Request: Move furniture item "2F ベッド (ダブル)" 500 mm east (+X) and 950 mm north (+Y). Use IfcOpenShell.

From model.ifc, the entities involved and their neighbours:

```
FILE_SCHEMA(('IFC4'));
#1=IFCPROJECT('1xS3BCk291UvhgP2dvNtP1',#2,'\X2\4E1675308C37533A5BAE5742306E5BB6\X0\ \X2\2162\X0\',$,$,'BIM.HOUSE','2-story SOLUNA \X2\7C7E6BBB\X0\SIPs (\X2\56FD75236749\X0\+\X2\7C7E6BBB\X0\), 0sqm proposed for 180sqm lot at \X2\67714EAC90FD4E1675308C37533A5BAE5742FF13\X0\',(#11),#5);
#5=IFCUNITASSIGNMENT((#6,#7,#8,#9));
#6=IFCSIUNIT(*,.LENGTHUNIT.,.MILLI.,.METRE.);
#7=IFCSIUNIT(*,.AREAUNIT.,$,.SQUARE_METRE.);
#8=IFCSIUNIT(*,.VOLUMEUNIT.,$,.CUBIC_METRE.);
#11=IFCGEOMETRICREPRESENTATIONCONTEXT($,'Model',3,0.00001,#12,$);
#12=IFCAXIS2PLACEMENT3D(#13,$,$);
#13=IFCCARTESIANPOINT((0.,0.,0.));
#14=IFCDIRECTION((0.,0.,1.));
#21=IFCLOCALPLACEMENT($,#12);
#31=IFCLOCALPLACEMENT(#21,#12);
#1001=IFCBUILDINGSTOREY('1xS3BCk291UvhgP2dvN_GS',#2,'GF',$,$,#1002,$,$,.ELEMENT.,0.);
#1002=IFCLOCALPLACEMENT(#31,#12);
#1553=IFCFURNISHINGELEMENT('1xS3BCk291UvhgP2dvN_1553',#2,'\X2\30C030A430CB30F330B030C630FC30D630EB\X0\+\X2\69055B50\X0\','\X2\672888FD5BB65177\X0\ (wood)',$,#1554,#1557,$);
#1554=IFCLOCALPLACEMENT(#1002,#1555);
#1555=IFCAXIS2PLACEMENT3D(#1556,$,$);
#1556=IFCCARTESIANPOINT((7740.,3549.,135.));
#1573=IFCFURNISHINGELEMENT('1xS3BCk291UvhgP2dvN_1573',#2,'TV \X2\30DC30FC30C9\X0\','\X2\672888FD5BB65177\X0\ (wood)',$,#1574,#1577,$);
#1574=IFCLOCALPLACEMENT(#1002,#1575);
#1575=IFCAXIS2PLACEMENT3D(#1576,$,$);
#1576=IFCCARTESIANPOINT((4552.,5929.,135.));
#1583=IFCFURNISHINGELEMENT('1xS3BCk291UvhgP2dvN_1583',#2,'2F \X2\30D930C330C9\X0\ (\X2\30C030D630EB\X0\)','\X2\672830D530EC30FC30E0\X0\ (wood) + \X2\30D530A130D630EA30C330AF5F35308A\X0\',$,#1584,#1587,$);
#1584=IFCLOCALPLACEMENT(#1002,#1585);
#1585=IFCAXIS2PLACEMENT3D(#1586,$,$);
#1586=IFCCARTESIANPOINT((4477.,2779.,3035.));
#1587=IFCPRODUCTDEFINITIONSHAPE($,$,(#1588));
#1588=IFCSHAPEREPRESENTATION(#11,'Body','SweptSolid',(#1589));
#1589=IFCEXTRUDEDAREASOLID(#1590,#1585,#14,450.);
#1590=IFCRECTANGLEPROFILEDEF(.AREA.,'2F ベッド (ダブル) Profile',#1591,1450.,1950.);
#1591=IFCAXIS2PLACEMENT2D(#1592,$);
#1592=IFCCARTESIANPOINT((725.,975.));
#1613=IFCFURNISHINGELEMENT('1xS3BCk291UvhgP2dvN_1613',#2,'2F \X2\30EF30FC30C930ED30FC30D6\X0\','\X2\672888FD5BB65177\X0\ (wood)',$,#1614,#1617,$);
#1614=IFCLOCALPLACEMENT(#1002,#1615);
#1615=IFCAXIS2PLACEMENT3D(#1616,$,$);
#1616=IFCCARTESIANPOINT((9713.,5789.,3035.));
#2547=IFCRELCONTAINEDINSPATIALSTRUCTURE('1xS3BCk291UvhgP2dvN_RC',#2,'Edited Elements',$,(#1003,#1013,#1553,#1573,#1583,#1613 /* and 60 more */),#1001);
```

```python
import ifcopenshell
import ifcopenshell.api.geometry
import ifcopenshell.util.placement

model = ifcopenshell.open("model.ifc")

item = model.by_guid("1xS3BCk291UvhgP2dvN_1583")
matrix = ifcopenshell.util.placement.get_local_placement(item.ObjectPlacement)
matrix[0, 3] += 500.0
matrix[1, 3] += 950.0
ifcopenshell.api.geometry.edit_object_placement(model, product=item, matrix=matrix, is_si=False)

print(ifcopenshell.util.placement.get_local_placement(item.ObjectPlacement).round(3) + 0.0)

model.write("model-out.ifc")
```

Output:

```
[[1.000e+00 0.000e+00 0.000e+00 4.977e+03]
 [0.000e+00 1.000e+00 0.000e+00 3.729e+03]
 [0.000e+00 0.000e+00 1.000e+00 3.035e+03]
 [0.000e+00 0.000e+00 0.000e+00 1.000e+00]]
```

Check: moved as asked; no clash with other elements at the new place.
